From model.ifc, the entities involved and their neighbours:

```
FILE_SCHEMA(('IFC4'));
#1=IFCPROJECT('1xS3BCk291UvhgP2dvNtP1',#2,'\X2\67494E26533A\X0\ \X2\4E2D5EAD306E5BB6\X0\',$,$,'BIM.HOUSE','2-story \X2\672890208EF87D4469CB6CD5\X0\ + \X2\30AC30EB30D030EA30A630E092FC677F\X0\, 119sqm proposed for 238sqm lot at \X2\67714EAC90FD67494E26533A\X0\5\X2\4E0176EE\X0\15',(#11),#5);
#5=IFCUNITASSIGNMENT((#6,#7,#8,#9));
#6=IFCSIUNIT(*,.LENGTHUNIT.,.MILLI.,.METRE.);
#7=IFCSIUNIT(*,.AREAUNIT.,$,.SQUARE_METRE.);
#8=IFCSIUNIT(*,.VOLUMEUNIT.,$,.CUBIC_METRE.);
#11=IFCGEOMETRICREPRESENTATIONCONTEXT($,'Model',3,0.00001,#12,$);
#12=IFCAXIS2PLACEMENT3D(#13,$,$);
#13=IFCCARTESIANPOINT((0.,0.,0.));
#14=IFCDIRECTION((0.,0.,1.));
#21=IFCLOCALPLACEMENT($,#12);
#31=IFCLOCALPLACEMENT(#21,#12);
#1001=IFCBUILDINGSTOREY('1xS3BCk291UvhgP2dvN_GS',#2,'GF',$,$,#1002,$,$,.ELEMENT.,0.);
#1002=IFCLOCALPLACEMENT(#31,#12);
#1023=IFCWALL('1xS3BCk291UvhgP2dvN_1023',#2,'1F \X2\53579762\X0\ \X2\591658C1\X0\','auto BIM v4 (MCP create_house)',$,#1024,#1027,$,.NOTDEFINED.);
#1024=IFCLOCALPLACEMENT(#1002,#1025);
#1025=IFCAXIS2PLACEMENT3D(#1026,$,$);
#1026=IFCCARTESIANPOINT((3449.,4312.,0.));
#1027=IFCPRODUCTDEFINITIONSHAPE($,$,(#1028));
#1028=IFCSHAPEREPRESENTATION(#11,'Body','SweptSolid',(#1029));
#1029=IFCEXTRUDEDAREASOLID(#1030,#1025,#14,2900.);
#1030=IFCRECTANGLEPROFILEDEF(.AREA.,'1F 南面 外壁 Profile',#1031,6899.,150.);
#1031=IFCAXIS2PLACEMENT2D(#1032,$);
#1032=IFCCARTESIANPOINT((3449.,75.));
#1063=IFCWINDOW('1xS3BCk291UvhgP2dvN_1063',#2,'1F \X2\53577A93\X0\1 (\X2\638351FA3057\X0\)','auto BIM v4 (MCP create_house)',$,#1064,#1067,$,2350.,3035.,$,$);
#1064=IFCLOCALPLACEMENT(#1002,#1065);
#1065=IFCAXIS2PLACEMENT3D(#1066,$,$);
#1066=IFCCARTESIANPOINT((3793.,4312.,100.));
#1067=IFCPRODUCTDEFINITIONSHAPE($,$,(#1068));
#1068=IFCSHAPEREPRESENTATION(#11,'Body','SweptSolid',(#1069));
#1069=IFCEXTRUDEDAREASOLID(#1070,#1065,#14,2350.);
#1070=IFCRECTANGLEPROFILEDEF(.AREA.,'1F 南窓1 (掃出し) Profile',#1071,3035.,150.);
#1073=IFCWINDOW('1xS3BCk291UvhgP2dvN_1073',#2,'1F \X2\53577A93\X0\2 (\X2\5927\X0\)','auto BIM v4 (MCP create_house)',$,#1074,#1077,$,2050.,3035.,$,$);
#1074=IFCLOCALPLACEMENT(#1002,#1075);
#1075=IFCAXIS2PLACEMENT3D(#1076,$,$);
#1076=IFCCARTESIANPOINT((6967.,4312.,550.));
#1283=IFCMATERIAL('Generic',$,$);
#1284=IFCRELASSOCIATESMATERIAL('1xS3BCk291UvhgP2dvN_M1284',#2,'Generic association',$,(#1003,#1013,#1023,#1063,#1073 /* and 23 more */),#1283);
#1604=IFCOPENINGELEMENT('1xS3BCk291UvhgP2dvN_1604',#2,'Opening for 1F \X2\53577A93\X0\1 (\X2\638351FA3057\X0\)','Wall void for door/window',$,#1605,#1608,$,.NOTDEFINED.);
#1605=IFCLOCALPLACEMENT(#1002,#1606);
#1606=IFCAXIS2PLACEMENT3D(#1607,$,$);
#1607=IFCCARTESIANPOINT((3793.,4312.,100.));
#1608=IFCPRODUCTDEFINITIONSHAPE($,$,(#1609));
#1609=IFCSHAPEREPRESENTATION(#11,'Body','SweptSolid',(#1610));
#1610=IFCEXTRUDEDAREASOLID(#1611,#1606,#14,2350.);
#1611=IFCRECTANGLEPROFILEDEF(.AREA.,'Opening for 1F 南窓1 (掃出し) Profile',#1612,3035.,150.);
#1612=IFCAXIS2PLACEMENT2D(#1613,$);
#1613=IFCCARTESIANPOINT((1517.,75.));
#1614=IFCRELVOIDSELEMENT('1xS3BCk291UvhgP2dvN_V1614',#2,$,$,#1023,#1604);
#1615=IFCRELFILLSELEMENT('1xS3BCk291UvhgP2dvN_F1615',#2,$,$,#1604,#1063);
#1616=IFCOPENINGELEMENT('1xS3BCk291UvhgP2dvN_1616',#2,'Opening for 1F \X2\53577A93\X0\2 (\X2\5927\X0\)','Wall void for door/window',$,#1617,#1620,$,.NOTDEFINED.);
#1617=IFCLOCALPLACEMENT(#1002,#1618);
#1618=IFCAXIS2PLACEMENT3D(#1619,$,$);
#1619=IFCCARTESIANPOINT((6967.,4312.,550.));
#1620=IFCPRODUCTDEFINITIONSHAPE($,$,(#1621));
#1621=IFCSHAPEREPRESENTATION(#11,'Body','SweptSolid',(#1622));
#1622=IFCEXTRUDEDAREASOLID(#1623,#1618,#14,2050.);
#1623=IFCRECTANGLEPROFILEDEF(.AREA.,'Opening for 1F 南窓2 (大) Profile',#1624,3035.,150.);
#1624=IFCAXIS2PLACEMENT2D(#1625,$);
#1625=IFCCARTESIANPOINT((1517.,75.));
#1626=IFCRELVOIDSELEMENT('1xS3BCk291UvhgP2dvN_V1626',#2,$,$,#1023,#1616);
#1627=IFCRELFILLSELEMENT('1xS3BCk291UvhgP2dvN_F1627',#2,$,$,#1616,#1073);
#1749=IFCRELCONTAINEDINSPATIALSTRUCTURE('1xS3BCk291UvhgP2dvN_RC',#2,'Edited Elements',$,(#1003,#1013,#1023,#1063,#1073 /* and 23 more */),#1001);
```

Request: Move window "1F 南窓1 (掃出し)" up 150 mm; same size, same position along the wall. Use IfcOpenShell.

```python
import numpy as np
import ifcopenshell
import ifcopenshell.api.geometry
import ifcopenshell.util.placement
import ifcopenshell.util.unit

model = ifcopenshell.open("model.ifc")
unit_scale = ifcopenshell.util.unit.calculate_unit_scale(model)

window = model.by_id(1063)
opening = window.FillsVoids[0].RelatingOpeningElement
dz = 0.15 / unit_scale

shift = np.array([0.0, 0.0, dz])
# The window is not placed relative to its opening, so move both.
for product in (opening, window):
    matrix = ifcopenshell.util.placement.get_local_placement(product.ObjectPlacement)
    matrix[:3, 3] += shift
    ifcopenshell.api.geometry.edit_object_placement(model, product=product, matrix=matrix, is_si=False)

print(f"moved by {dz * unit_scale:+.3f} m")

model.write("model-out.ifc")
```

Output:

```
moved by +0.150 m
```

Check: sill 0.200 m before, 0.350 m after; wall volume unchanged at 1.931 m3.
